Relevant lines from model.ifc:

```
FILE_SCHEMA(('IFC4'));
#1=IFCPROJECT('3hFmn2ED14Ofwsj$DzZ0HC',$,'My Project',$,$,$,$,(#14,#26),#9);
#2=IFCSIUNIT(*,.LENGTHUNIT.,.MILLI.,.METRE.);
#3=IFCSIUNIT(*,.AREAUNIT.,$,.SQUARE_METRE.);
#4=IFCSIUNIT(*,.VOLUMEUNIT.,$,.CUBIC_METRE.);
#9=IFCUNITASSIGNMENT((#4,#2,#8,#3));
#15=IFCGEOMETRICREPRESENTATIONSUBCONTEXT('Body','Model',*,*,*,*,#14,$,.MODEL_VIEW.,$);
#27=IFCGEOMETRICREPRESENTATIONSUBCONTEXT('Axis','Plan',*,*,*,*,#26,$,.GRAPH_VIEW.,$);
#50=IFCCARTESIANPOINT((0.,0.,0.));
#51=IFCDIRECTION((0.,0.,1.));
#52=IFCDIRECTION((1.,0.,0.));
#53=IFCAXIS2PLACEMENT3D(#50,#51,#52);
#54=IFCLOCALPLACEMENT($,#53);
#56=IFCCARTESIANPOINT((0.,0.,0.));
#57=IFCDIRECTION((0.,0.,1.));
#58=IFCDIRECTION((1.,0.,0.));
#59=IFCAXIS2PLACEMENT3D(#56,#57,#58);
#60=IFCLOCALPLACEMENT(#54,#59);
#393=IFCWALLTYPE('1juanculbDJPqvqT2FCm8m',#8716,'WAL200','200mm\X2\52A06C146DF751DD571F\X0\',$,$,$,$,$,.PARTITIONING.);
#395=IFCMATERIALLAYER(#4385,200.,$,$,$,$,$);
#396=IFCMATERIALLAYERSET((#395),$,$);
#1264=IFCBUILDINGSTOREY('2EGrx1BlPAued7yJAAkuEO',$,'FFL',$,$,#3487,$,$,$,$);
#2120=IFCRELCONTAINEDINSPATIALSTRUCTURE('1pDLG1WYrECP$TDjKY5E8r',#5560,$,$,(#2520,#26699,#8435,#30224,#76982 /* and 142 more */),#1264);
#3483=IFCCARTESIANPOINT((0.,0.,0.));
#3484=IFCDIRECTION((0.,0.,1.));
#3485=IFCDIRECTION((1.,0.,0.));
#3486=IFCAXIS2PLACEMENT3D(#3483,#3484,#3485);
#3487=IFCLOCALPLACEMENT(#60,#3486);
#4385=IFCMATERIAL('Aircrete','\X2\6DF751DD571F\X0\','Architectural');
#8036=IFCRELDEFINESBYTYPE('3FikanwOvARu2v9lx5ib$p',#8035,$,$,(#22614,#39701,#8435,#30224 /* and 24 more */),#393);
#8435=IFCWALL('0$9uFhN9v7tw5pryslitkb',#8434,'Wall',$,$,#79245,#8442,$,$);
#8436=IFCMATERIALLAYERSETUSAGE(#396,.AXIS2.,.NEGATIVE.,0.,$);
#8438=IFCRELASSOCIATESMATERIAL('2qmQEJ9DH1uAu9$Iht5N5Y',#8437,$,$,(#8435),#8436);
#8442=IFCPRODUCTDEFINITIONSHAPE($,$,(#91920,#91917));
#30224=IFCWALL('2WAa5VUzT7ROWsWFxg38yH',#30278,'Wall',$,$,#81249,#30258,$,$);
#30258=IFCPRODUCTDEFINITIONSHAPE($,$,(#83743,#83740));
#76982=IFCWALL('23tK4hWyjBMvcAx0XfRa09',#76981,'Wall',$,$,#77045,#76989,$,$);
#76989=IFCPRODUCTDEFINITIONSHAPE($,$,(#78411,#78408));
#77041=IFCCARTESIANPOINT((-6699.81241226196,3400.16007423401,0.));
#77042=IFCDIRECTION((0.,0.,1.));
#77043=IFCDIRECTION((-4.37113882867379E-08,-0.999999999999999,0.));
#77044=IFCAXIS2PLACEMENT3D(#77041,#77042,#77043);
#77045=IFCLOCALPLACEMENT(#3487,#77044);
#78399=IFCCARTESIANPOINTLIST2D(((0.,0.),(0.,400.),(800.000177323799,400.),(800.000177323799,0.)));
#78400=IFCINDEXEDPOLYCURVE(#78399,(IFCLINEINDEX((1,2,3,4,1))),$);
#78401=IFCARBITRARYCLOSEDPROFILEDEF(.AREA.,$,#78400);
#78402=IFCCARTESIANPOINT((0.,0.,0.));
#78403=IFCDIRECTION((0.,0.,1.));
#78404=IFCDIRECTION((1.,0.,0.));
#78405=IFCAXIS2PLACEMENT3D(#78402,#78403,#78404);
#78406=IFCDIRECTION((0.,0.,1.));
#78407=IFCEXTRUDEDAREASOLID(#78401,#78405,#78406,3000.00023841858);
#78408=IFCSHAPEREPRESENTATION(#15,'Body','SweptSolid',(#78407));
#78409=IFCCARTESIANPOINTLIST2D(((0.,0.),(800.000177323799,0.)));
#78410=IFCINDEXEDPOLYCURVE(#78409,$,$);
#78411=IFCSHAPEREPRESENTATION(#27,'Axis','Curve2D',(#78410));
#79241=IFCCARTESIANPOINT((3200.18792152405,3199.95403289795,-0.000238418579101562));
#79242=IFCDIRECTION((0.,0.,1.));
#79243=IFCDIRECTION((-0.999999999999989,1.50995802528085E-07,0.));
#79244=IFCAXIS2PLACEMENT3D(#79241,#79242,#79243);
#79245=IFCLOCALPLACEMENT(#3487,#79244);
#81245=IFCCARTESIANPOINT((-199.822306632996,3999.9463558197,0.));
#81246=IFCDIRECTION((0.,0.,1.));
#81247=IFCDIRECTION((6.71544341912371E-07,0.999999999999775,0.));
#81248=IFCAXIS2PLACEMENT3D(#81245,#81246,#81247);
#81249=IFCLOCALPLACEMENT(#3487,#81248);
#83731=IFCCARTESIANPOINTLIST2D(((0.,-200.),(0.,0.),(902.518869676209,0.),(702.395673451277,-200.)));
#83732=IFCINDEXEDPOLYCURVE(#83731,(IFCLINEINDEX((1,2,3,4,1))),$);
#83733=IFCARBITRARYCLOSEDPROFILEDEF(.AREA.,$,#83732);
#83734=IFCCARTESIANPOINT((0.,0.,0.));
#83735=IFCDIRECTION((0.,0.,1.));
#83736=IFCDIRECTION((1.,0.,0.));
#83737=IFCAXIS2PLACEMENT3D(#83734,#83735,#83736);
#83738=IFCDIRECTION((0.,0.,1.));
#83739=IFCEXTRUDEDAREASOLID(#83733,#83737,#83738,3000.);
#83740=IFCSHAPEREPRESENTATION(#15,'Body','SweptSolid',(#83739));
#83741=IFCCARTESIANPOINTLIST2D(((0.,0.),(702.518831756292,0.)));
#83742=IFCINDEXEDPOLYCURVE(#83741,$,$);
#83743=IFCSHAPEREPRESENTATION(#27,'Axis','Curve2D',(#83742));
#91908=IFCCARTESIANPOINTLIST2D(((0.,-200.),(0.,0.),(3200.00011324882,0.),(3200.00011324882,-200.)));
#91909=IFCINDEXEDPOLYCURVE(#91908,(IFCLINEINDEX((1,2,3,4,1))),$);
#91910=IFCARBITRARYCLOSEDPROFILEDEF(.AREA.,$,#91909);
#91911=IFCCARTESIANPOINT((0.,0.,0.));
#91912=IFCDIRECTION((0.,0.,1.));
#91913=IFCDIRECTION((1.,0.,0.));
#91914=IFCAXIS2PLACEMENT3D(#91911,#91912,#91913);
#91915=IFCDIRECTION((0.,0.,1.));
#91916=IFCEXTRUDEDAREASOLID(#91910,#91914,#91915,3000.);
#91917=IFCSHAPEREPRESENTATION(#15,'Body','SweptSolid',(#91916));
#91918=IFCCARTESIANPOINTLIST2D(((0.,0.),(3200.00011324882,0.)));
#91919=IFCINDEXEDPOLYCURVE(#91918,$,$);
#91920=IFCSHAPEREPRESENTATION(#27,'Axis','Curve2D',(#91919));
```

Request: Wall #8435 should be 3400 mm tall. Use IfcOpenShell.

```python
import ifcopenshell
import ifcopenshell.geom
import ifcopenshell.util.representation
import ifcopenshell.util.shape

model = ifcopenshell.open("model.ifc")
settings = ifcopenshell.geom.settings()


def volume(element):
    """Net volume in cubic metres, openings subtracted."""
    shape = ifcopenshell.geom.create_shape(settings, element)
    return ifcopenshell.util.shape.get_volume(shape.geometry)


wall = model.by_id(8435)
before = volume(wall)

body = ifcopenshell.util.representation.get_representation(wall, "Model", "Body")
solid = body.Items[0]
old_height = solid.Depth
solid.Depth = 3400.0
after = volume(wall)

print(f"height {old_height:g} -> {solid.Depth:g}, volume {before:.3f} -> {after:.3f} m3")

model.write("model_v2.ifc")
```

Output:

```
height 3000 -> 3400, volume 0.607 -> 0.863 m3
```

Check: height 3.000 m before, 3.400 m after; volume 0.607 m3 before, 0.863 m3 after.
